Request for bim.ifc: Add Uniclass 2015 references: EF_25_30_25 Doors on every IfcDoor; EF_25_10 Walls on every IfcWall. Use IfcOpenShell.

First a look at what the model holds.

```python
import ifcopenshell

model = ifcopenshell.open("bim.ifc")
print(model.schema)
print("classifications:", [c.Name for c in model.by_type("IfcClassification")])
for ifc_class in ("IfcDoor", "IfcRoof", "IfcStair", "IfcWall", "IfcWindow"):
    print(ifc_class, len(model.by_type(ifc_class)))
```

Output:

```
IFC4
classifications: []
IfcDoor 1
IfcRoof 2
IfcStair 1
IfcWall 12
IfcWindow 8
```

```python
import ifcopenshell
import ifcopenshell.api.classification

model = ifcopenshell.open("bim.ifc")

system = ifcopenshell.api.classification.add_classification(model, classification="Uniclass 2015")

codes = {
    "IfcDoor": ("EF_25_30_25", "Doors"),
    "IfcWall": ("EF_25_10", "Walls"),
}
for ifc_class, (code, name) in codes.items():
    products = model.by_type(ifc_class)
    ifcopenshell.api.classification.add_reference(
        model, products=products, classification=system, identification=code, name=name
    )
    print(code, len(products))

model.write("bim-out.ifc")
```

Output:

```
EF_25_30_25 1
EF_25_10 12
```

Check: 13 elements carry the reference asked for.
